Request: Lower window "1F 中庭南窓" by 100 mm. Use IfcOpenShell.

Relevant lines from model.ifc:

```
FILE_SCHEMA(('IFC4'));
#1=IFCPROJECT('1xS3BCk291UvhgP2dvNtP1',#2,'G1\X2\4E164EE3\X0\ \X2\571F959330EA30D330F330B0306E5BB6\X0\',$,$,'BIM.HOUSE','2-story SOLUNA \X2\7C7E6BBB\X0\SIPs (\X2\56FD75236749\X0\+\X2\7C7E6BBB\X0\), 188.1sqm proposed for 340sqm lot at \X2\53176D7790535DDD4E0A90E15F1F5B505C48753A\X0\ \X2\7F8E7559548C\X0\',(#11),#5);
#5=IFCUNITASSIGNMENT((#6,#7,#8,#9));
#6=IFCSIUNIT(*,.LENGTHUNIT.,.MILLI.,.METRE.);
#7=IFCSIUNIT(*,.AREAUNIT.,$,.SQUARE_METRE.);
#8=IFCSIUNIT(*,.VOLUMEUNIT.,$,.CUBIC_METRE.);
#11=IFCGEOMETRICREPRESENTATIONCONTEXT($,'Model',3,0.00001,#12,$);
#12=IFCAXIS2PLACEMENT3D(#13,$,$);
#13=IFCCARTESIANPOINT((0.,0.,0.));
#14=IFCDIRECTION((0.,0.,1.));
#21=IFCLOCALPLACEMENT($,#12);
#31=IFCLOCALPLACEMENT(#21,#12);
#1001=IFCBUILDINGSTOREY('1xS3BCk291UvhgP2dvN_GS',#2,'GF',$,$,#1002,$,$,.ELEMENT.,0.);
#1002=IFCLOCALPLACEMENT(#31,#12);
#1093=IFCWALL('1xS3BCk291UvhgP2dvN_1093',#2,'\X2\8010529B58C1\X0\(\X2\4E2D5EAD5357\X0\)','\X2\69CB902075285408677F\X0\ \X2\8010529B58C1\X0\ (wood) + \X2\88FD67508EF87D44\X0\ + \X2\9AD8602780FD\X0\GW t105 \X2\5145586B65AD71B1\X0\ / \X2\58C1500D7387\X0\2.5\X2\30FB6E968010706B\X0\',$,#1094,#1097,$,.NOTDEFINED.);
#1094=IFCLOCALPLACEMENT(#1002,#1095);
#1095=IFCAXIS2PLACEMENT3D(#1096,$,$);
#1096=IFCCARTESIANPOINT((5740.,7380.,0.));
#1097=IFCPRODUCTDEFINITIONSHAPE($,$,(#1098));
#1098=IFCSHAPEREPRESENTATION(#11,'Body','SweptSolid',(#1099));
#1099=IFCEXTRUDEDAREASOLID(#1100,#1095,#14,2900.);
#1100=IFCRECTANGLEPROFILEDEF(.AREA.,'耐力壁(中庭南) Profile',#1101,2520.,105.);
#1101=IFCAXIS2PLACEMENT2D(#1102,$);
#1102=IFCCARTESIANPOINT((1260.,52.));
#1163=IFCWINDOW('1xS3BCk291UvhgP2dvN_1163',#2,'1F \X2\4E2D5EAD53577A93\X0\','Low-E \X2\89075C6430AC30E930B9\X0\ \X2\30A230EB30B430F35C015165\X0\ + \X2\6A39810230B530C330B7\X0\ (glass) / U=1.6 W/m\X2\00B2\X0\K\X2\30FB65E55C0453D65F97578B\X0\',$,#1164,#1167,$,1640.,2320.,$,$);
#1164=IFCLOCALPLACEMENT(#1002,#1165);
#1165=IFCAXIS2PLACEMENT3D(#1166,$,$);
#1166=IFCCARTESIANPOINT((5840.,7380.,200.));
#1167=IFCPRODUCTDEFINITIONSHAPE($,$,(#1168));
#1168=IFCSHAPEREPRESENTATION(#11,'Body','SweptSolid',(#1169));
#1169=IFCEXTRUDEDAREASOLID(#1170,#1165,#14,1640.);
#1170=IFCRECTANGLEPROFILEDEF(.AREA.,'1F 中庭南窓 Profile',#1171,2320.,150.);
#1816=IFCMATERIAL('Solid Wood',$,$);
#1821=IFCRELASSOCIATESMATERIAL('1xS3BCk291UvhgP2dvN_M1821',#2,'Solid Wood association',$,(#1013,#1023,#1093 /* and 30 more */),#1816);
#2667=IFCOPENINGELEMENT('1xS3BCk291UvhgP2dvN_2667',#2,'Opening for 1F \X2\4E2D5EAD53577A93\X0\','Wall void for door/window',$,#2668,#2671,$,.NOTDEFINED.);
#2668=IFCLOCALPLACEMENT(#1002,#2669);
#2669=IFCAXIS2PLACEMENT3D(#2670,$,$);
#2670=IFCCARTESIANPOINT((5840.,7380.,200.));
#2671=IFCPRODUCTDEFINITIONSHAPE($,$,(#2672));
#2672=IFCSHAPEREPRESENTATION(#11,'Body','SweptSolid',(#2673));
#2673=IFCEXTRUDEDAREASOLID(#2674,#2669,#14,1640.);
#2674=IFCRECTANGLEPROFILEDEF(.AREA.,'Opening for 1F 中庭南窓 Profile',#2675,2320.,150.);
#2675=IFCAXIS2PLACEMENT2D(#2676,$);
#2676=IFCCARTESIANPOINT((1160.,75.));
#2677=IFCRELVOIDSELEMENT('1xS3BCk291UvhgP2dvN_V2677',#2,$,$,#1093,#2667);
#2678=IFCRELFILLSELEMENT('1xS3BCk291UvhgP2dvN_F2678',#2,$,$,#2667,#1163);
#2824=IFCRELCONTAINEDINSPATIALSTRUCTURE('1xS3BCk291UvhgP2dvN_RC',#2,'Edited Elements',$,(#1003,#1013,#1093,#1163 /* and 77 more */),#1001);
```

```python
import numpy as np
import ifcopenshell
import ifcopenshell.api.geometry
import ifcopenshell.util.placement
import ifcopenshell.util.unit

model = ifcopenshell.open("model.ifc")
unit_scale = ifcopenshell.util.unit.calculate_unit_scale(model)

window = model.by_guid("1xS3BCk291UvhgP2dvN_1163")
opening = window.FillsVoids[0].RelatingOpeningElement
dz = -0.1 / unit_scale

shift = np.array([0.0, 0.0, dz])
# The window is not placed relative to its opening, so move both.
for product in (opening, window):
    matrix = ifcopenshell.util.placement.get_local_placement(product.ObjectPlacement)
    matrix[:3, 3] += shift
    ifcopenshell.api.geometry.edit_object_placement(model, product=product, matrix=matrix, is_si=False)

print(f"moved by {dz * unit_scale:+.3f} m")

model.write("model_v2.ifc")
```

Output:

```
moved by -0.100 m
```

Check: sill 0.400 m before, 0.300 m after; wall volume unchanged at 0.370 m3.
